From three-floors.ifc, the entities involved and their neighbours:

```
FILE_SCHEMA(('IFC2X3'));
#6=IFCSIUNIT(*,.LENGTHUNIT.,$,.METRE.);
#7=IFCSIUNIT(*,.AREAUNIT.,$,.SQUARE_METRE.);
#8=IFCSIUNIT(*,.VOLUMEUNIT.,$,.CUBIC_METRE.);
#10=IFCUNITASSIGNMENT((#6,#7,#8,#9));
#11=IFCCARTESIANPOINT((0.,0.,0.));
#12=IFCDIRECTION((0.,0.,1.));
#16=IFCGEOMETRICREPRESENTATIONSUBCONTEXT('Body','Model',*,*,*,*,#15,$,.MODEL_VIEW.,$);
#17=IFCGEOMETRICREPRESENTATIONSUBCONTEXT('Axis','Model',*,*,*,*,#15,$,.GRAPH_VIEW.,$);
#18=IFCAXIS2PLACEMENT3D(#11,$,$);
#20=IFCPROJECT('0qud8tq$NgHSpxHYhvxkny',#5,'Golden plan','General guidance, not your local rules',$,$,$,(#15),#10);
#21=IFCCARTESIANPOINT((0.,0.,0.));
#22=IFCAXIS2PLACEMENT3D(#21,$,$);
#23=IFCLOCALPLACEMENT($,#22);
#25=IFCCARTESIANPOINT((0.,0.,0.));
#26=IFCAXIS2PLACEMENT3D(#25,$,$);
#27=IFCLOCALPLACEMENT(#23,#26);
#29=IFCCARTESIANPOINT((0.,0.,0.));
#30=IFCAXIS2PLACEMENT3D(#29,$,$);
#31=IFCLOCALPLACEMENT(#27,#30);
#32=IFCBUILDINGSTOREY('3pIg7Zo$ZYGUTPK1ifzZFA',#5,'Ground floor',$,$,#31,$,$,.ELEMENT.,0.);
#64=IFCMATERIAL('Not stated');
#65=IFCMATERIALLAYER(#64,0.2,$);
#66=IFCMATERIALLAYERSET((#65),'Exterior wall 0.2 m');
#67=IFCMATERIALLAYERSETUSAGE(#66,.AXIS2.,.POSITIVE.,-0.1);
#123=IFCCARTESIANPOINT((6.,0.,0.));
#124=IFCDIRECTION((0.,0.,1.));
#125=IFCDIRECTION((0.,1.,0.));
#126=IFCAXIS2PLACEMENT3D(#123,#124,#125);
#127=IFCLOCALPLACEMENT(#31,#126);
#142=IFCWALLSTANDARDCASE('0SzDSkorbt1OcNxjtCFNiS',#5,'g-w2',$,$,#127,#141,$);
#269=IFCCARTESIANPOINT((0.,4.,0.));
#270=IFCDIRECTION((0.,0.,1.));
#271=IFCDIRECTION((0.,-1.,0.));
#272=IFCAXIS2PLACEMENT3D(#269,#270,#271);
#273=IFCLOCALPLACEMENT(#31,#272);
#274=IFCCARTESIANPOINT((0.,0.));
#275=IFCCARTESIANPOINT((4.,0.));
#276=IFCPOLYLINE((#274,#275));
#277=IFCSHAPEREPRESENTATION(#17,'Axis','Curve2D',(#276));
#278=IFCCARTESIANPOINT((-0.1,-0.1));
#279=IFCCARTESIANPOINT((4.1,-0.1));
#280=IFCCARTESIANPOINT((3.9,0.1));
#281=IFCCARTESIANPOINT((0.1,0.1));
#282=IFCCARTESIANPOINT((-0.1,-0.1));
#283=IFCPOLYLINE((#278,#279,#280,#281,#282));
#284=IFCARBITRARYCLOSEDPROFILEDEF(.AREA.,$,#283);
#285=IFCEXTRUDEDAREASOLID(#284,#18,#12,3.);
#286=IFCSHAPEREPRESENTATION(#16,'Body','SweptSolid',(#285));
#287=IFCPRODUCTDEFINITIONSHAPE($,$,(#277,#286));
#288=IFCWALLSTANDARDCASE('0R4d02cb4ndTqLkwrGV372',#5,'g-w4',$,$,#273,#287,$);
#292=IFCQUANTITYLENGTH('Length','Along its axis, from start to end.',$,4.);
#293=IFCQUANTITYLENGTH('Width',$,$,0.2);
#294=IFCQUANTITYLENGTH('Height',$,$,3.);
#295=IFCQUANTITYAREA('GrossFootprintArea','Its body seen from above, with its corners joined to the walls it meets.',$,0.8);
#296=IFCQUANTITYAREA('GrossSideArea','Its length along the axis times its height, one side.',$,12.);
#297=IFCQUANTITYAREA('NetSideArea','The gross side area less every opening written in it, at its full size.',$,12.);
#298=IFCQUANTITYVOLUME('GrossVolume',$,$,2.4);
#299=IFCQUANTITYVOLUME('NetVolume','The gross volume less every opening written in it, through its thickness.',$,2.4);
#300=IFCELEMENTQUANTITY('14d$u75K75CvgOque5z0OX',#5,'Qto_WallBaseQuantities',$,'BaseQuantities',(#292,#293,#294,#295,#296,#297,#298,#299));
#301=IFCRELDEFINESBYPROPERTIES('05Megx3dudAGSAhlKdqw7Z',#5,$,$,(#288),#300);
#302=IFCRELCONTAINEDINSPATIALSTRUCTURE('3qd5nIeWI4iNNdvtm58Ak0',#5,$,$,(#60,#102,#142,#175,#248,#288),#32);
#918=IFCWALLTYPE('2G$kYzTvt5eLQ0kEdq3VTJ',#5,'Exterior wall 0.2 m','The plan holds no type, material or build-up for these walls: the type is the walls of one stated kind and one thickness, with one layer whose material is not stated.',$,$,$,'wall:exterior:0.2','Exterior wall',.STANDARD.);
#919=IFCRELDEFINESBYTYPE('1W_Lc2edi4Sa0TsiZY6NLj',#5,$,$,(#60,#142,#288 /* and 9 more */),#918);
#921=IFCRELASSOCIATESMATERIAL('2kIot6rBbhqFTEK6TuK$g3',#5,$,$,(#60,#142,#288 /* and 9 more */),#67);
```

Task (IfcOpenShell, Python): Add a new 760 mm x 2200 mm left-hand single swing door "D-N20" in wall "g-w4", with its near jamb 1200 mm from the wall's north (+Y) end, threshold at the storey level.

```python
import numpy as np
import ifcopenshell
import ifcopenshell.api.feature
import ifcopenshell.api.geometry
import ifcopenshell.api.pset
import ifcopenshell.api.root
import ifcopenshell.api.spatial
import ifcopenshell.api.type
import ifcopenshell.geom
import ifcopenshell.util.element
import ifcopenshell.util.placement
import ifcopenshell.util.representation
import ifcopenshell.util.shape
import ifcopenshell.util.unit

model = ifcopenshell.open("three-floors.ifc")
unit_scale = ifcopenshell.util.unit.calculate_unit_scale(model)
area_scale = ifcopenshell.util.unit.calculate_unit_scale(model, "AREAUNIT")
volume_scale = ifcopenshell.util.unit.calculate_unit_scale(model, "VOLUMEUNIT")
settings = ifcopenshell.geom.settings()


def volume(element):
    """Net volume in cubic metres, openings subtracted."""
    shape = ifcopenshell.geom.create_shape(settings, element)
    return ifcopenshell.util.shape.get_volume(shape.geometry)


wall = model.by_guid("0R4d02cb4ndTqLkwrGV372")
storey = ifcopenshell.util.element.get_container(wall, ifc_class="IfcBuildingStorey")
context = ifcopenshell.util.representation.get_context(model, "Model", "Body", "MODEL_VIEW")
before = volume(wall)

width, height, from_end, sill = 0.76, 2.2, 1.2, 0.0  # metres

# The wall runs along its own X axis, and the end named is its -X end.
wall_shape = ifcopenshell.geom.create_shape(settings, wall)
x, y, z = ifcopenshell.util.shape.get_vertices(wall_shape.geometry).T
start = x.min() + from_end
face, thickness = float(y.min()), float(y.max() - y.min())
wall_matrix = ifcopenshell.util.placement.get_local_placement(wall.ObjectPlacement)
level = ifcopenshell.util.placement.get_local_placement(storey.ObjectPlacement)[2, 3]


def in_wall(x, y):
    """Placement at x, y metres in the wall's axes, at sill height."""
    matrix = wall_matrix.copy()
    matrix[:, 3] = wall_matrix @ np.array([x / unit_scale, y / unit_scale, 0.0, 1.0])
    matrix[2, 3] = level + sill / unit_scale
    return matrix


# Opening: a box that overshoots both wall faces by 50 mm.
opening = ifcopenshell.api.root.create_entity(model, ifc_class="IfcOpeningElement")
box = ifcopenshell.api.geometry.add_wall_representation(
    model, context=context, length=width, height=height, thickness=thickness + 0.1
)
ifcopenshell.api.geometry.assign_representation(model, product=opening, representation=box)
ifcopenshell.api.geometry.edit_object_placement(model, product=opening, matrix=in_wall(start, face - 0.05), is_si=False)
ifcopenshell.api.feature.add_feature(model, feature=opening, element=wall)

door = ifcopenshell.api.root.create_entity(model, ifc_class="IfcDoor", name="D-N20")
door.OverallWidth, door.OverallHeight = width / unit_scale, height / unit_scale
body = ifcopenshell.api.geometry.add_door_representation(
    model,
    context=context,
    overall_width=door.OverallWidth,
    overall_height=door.OverallHeight,
    operation_type="SINGLE_SWING_LEFT",
    lining_properties={"LiningDepth": thickness / unit_scale, "ThresholdDepth": thickness / unit_scale},
)
ifcopenshell.api.geometry.assign_representation(model, product=door, representation=body)
ifcopenshell.api.spatial.assign_container(model, products=[door], relating_structure=storey)
fills = ifcopenshell.api.feature.add_filling(model, opening=opening, element=door)
fills.OwnerHistory = door.OwnerHistory  # required in IFC2X3

# IFC2X3 keeps the operation on the door style.
style = ifcopenshell.api.root.create_entity(model, ifc_class="IfcDoorStyle", name="D-N20")
style.OperationType, style.ConstructionType = "SINGLE_SWING_LEFT", "NOTDEFINED"
style.ParameterTakesPrecedence = style.Sizeable = False
ifcopenshell.api.type.assign_type(model, related_objects=[door], relating_type=style)

# The lining spans the wall, so the door starts at the wall face.
ifcopenshell.api.geometry.edit_object_placement(model, product=door, matrix=in_wall(start, face), is_si=False)

after = volume(wall)

# Update the wall's stored quantities.
qto = model.by_id(ifcopenshell.util.element.get_pset(wall, "Qto_WallBaseQuantities", should_inherit=False)["id"])
ifcopenshell.api.pset.edit_qto(model, qto=qto, properties={
    "NetSideArea": after / thickness / area_scale,
    "NetVolume": after / volume_scale,
})

print(f"wall volume {before:.3f} -> {after:.3f} m3")

model.write("three-floors-out.ifc")
```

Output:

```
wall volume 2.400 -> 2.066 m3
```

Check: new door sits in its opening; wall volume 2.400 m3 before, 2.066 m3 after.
